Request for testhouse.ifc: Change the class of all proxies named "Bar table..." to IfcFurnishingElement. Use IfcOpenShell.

First a look at what the model holds.

```python
import re

import ifcopenshell

model = ifcopenshell.open("testhouse.ifc")
print(model.schema)
seen = {}
for e in model.by_type("IfcBuildingElementProxy"):
    name = re.sub(r":\d+(:\d+)?$", "", e.Name or "")  # drop the element id that some exporters append
    seen[name] = seen.get(name, 0) + 1
for name, count in sorted(seen.items()):
    print(count, "x", name)
```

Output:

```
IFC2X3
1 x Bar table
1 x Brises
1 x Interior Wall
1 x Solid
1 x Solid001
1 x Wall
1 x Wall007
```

```python
import ifcopenshell
import ifcopenshell.api.root

model = ifcopenshell.open("testhouse.ifc")

proxies = [e.id() for e in model.by_type("IfcBuildingElementProxy") if (e.Name or "").startswith("Bar table")]
for step_id in proxies:
    proxy = model.by_id(step_id)
    ifcopenshell.api.root.reassign_class(model, product=proxy, ifc_class="IfcFurnishingElement")

print(sum(model.by_id(i).is_a("IfcFurnishingElement") for i in proxies), "reclassified")

model.write("testhouse_rev.ifc")
```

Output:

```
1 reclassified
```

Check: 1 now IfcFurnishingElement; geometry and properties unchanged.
